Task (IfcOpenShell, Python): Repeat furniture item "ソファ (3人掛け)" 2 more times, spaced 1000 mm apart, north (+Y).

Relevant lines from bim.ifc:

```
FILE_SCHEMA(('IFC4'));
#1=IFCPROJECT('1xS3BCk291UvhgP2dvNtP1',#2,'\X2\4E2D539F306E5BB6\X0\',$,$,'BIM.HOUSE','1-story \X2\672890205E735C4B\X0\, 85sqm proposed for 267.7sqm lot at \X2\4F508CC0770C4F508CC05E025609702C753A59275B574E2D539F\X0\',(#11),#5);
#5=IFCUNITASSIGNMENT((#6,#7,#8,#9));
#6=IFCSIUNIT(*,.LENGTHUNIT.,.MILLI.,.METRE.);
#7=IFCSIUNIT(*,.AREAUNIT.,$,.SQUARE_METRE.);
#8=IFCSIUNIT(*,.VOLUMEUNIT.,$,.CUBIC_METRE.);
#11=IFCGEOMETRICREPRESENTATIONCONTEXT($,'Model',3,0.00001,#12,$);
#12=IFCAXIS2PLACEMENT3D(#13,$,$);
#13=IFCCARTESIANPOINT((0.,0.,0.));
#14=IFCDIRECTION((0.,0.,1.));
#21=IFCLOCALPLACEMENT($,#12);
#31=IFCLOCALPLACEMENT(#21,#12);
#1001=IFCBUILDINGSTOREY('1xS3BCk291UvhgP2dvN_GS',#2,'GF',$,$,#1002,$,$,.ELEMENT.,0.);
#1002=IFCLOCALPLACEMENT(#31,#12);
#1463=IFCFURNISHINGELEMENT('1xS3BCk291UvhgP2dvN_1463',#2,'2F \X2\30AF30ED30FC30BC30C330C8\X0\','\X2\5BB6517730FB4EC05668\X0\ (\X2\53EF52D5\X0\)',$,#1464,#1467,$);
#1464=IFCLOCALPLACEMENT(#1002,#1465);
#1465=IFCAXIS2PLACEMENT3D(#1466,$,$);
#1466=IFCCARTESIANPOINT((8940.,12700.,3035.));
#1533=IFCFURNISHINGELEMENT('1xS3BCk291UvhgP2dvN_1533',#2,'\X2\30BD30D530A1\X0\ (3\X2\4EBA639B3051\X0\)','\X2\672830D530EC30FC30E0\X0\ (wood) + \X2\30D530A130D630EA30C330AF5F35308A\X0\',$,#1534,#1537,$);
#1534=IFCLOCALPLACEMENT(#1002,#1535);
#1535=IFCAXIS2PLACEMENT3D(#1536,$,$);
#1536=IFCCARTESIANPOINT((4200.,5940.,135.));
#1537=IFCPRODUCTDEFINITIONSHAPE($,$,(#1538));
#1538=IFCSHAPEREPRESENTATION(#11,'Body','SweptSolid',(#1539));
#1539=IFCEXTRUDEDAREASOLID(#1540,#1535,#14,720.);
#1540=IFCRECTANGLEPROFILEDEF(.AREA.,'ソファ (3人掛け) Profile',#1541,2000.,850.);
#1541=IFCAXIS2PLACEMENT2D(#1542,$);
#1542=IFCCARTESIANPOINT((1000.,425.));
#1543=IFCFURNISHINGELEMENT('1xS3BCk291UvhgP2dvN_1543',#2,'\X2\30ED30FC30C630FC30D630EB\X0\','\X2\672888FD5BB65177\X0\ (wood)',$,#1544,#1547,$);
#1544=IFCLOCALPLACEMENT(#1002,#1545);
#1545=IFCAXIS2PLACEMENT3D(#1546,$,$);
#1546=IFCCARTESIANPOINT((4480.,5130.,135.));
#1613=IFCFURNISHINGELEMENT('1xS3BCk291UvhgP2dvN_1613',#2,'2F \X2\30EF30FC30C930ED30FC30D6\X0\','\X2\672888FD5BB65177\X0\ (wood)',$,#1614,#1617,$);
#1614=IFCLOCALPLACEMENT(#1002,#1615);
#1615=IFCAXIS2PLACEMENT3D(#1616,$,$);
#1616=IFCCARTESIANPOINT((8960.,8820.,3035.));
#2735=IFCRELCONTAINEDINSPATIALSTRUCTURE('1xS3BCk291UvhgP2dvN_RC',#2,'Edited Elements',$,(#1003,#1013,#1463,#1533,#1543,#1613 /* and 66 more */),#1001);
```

```python
import numpy as np
import ifcopenshell
import ifcopenshell.api.geometry
import ifcopenshell.api.root
import ifcopenshell.util.element
import ifcopenshell.util.placement
import ifcopenshell.util.unit

model = ifcopenshell.open("bim.ifc")
unit_scale = ifcopenshell.util.unit.calculate_unit_scale(model)


def reuse_history(source, copy):
    """copy_class also copies each property set's owner history, people and application; keep the originals."""
    for rel in copy.IsDefinedBy:
        if rel.is_a("IfcRelDefinesByProperties") and (history := rel.RelatingPropertyDefinition.OwnerHistory):
            rel.RelatingPropertyDefinition.OwnerHistory = source.OwnerHistory
            ifcopenshell.util.element.remove_deep2(model, history)


source = model.by_guid("1xS3BCk291UvhgP2dvN_1533")
base = ifcopenshell.util.placement.get_local_placement(source.ObjectPlacement)
step = np.array([0.0, 1.0, 0.0]) * 1 / unit_scale

for i in range(1, 3):
    copy = ifcopenshell.api.root.copy_class(model, product=source)
    copy.Representation = ifcopenshell.util.element.copy_deep(
        model, source.Representation, exclude=["IfcGeometricRepresentationContext", "IfcRepresentationMap"]
    )
    reuse_history(source, copy)
    matrix = base.copy()
    matrix[:3, 3] += i * step
    print("added at", matrix[:3, 3].round(3) + 0.0)
    ifcopenshell.api.geometry.edit_object_placement(model, product=copy, matrix=matrix, is_si=False)

model.write("bim_updated.ifc")
```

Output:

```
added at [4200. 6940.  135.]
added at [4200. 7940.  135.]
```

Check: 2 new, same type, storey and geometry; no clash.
